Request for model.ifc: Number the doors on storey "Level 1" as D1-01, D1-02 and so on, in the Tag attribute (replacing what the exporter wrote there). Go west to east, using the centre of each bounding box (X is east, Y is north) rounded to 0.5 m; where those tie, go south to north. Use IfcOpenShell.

First a look at what the model holds.

```python
import ifcopenshell
import ifcopenshell.util.element
import ifcopenshell.util.placement

model = ifcopenshell.open("model.ifc")
print(model.schema)
storey = next(s for s in model.by_type("IfcBuildingStorey") if s.Name == "Level 1")
doors = [e for e in ifcopenshell.util.element.get_decomposition(storey) if e.is_a("IfcDoor")]
for e in sorted(doors, key=lambda e: e.id()):
    origin = ifcopenshell.util.placement.get_local_placement(e.ObjectPlacement)[:3, 3]
    print(e.id(), e.Tag, e.Name, origin.round(2) + 0.0, sep=" | ")
```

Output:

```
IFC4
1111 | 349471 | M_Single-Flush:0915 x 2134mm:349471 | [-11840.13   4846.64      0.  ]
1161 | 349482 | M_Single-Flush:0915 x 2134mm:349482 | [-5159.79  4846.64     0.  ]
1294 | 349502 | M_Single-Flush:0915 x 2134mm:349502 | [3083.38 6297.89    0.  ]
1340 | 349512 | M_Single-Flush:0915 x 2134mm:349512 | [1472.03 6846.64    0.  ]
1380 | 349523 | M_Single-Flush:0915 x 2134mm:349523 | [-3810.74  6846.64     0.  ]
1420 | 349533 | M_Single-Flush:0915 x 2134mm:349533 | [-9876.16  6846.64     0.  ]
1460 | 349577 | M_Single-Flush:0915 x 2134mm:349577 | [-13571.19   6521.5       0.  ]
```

```python
import ifcopenshell
import ifcopenshell.geom
import ifcopenshell.util.element
import ifcopenshell.util.shape

model = ifcopenshell.open("model.ifc")
settings = ifcopenshell.geom.settings()
settings.set("use-world-coords", True)


def centre(element):
    shape = ifcopenshell.geom.create_shape(settings, element)
    return ifcopenshell.util.shape.get_bbox_centroid(shape.geometry)


storey = next(s for s in model.by_type("IfcBuildingStorey") if s.Name == "Level 1")
doors = [e for e in ifcopenshell.util.element.get_decomposition(storey) if e.is_a("IfcDoor")]

# Insertion points can sit at a corner or the storey origin, so sort by the geometry (in metres).
centres = {e: centre(e) for e in doors}
doors.sort(key=lambda e: (round(centres[e][0] / 0.5), centres[e][1]))

for i, e in enumerate(doors, start=1):
    number = f"D1-{i:02d}"
    e.Tag = number
    print(e.id(), number)

model.write("model-out.ifc")
```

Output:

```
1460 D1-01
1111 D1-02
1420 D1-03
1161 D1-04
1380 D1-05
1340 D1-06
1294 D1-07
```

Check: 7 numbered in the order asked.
